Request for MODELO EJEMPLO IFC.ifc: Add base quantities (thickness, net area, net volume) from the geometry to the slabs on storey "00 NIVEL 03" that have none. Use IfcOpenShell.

First a look at what the model holds.

```python
import ifcopenshell
import ifcopenshell.util.element
import ifcopenshell.util.unit

model = ifcopenshell.open("MODELO EJEMPLO IFC.ifc")
print(model.schema)
for unit_type in ("LENGTHUNIT", "AREAUNIT", "VOLUMEUNIT"):
    print(unit_type, ifcopenshell.util.unit.calculate_unit_scale(model, unit_type))
storey = next(s for s in model.by_type("IfcBuildingStorey") if s.Name == "00 NIVEL 03")
slabs = [e for e in ifcopenshell.util.element.get_decomposition(storey) if e.is_a("IfcSlab")]
for e in sorted(slabs, key=lambda e: e.id()):
    print(e.id(), e.is_a(), e.Name, list(ifcopenshell.util.element.get_psets(e, qtos_only=True)), sep=" | ")
```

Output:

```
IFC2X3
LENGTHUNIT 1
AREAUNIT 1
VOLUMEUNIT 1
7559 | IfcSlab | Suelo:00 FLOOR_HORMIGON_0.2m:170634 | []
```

```python
import ifcopenshell
import ifcopenshell.api.pset
import ifcopenshell.geom
import ifcopenshell.util.element
import ifcopenshell.util.shape
import ifcopenshell.util.unit

model = ifcopenshell.open("MODELO EJEMPLO IFC.ifc")
unit_scale = ifcopenshell.util.unit.calculate_unit_scale(model)
area_scale = ifcopenshell.util.unit.calculate_unit_scale(model, "AREAUNIT")
volume_scale = ifcopenshell.util.unit.calculate_unit_scale(model, "VOLUMEUNIT")
settings = ifcopenshell.geom.settings()

storey = next(s for s in model.by_type("IfcBuildingStorey") if s.Name == "00 NIVEL 03")
slabs = [e for e in ifcopenshell.util.element.get_decomposition(storey) if e.is_a("IfcSlab")]

for e in sorted(slabs, key=lambda e: e.id()):
    if ifcopenshell.util.element.get_psets(e, qtos_only=True, should_inherit=False):
        continue
    # Geometry comes back in metres, in the element's own axes.
    shape = ifcopenshell.geom.create_shape(settings, e)
    values = {
        "Width": ifcopenshell.util.shape.get_z(shape.geometry) / unit_scale,
        "NetArea": ifcopenshell.util.shape.get_footprint_area(shape.geometry) / area_scale,
        "NetVolume": ifcopenshell.util.shape.get_volume(shape.geometry) / volume_scale,
    }
    qto = ifcopenshell.api.pset.add_qto(model, product=e, name="BaseQuantities")
    ifcopenshell.api.pset.edit_qto(model, qto=qto, properties=values)
    print(e.id(), {k: round(v, 3) for k, v in values.items()})

model.write("MODELO EJEMPLO IFC_updated.ifc")
```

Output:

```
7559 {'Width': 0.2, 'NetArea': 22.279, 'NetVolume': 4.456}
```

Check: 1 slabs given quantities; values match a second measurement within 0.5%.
